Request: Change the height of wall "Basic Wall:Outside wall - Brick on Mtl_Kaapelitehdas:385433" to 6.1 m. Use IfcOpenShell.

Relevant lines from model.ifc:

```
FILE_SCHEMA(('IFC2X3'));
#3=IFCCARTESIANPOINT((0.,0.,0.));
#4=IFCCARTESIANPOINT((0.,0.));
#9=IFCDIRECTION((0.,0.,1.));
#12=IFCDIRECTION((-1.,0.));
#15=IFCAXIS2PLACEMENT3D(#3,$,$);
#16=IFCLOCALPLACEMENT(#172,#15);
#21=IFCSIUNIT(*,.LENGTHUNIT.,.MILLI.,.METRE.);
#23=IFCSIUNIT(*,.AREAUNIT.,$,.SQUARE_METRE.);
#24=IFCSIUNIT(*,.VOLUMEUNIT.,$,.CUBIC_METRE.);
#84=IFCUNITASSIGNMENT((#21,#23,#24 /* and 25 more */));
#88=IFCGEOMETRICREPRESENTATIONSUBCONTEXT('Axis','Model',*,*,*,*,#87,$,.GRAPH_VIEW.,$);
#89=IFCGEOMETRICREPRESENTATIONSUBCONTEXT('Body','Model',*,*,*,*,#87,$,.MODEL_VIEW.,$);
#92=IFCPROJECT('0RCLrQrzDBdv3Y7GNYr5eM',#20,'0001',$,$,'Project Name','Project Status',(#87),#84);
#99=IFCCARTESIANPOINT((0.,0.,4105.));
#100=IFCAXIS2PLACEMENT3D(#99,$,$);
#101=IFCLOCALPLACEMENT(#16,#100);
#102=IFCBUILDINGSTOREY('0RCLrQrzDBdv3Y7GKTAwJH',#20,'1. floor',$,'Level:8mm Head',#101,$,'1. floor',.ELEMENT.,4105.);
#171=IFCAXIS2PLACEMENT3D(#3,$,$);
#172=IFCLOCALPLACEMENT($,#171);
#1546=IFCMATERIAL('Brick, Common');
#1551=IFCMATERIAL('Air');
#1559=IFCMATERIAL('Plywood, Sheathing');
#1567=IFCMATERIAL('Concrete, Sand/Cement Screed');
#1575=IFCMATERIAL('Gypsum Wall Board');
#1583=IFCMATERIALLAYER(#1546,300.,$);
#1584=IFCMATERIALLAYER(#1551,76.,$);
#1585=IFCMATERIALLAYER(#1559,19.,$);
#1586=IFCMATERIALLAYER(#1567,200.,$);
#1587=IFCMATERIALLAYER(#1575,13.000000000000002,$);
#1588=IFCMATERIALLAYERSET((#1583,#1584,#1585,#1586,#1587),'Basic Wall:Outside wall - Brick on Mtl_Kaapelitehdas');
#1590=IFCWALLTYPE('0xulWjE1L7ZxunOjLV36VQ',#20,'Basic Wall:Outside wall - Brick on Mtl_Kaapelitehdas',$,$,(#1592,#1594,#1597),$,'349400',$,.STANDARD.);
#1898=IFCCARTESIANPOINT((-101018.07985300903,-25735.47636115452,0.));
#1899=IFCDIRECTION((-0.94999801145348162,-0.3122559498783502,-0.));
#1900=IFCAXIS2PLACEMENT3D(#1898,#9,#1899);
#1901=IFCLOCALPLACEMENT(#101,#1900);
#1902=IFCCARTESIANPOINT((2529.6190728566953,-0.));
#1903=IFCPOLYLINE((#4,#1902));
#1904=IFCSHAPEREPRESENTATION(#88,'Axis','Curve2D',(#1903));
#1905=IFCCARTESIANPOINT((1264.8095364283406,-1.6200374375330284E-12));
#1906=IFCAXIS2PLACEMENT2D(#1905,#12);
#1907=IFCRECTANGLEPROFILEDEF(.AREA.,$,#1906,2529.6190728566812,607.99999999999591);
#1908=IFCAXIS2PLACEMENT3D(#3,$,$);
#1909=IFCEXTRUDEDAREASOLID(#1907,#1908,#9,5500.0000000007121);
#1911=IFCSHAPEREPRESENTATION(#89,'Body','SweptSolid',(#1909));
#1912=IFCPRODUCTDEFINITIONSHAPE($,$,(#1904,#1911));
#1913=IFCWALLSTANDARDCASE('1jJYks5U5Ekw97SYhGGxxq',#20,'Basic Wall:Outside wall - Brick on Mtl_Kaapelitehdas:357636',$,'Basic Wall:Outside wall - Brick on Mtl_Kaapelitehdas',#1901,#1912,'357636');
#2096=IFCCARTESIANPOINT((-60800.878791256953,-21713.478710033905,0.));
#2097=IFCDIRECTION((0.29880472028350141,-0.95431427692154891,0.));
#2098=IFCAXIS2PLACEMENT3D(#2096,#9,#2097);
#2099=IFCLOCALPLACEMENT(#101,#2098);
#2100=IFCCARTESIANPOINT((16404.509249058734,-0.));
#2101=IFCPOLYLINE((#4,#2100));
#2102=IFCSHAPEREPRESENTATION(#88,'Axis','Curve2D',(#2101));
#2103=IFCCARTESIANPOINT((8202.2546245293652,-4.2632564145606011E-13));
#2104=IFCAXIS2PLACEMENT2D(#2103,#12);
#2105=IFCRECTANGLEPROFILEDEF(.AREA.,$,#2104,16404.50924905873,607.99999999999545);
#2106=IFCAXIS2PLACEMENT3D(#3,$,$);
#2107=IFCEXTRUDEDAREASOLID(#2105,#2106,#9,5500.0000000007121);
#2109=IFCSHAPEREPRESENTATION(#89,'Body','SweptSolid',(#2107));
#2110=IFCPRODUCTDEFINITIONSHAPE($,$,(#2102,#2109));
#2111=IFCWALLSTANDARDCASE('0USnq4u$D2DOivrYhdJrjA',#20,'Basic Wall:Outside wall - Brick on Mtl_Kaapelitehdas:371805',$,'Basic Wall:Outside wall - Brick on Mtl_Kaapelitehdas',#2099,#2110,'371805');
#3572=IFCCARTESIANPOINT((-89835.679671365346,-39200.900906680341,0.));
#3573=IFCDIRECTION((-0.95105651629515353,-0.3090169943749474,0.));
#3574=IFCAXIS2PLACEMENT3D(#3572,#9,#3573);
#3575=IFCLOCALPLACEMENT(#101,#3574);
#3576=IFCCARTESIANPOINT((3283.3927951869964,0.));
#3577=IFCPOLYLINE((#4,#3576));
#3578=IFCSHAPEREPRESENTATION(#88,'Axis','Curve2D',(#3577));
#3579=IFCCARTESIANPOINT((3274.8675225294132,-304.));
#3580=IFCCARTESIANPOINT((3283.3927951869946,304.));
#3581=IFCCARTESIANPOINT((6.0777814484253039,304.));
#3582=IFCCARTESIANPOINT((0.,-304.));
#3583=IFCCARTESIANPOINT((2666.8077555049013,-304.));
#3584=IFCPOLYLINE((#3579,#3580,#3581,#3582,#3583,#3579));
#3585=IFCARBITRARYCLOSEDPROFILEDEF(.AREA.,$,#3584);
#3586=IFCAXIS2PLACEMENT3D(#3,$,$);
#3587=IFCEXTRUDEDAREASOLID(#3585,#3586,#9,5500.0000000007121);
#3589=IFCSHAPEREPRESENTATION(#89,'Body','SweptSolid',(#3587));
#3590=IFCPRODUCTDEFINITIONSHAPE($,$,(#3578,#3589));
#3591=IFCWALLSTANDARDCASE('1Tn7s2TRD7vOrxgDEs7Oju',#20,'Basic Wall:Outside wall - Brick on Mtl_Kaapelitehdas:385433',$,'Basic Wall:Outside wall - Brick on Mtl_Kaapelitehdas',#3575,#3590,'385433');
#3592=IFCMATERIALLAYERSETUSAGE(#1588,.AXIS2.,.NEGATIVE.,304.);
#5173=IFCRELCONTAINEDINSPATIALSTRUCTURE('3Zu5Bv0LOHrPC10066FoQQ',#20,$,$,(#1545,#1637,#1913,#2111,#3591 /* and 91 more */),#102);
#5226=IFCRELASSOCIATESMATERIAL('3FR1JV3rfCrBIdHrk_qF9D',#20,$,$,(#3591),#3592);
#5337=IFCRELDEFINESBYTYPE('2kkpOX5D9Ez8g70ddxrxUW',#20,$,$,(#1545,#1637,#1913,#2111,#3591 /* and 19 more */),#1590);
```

```python
import ifcopenshell
import ifcopenshell.geom
import ifcopenshell.util.representation
import ifcopenshell.util.shape
import ifcopenshell.util.unit

model = ifcopenshell.open("model.ifc")
unit_scale = ifcopenshell.util.unit.calculate_unit_scale(model)
settings = ifcopenshell.geom.settings()


def volume(element):
    """Net volume in cubic metres, openings subtracted."""
    shape = ifcopenshell.geom.create_shape(settings, element)
    return ifcopenshell.util.shape.get_volume(shape.geometry)


wall = model.by_guid("1Tn7s2TRD7vOrxgDEs7Oju")
before = volume(wall)

body = ifcopenshell.util.representation.get_representation(wall, "Model", "Body")
solid = body.Items[0]
old_height = solid.Depth
solid.Depth = 6.1 / unit_scale
after = volume(wall)

print(f"height {old_height:g} -> {solid.Depth:g}, volume {before:.3f} -> {after:.3f} m3")

model.write("model_v2.ifc")
```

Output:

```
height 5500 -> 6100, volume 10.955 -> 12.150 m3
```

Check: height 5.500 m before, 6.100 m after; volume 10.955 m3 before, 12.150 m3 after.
